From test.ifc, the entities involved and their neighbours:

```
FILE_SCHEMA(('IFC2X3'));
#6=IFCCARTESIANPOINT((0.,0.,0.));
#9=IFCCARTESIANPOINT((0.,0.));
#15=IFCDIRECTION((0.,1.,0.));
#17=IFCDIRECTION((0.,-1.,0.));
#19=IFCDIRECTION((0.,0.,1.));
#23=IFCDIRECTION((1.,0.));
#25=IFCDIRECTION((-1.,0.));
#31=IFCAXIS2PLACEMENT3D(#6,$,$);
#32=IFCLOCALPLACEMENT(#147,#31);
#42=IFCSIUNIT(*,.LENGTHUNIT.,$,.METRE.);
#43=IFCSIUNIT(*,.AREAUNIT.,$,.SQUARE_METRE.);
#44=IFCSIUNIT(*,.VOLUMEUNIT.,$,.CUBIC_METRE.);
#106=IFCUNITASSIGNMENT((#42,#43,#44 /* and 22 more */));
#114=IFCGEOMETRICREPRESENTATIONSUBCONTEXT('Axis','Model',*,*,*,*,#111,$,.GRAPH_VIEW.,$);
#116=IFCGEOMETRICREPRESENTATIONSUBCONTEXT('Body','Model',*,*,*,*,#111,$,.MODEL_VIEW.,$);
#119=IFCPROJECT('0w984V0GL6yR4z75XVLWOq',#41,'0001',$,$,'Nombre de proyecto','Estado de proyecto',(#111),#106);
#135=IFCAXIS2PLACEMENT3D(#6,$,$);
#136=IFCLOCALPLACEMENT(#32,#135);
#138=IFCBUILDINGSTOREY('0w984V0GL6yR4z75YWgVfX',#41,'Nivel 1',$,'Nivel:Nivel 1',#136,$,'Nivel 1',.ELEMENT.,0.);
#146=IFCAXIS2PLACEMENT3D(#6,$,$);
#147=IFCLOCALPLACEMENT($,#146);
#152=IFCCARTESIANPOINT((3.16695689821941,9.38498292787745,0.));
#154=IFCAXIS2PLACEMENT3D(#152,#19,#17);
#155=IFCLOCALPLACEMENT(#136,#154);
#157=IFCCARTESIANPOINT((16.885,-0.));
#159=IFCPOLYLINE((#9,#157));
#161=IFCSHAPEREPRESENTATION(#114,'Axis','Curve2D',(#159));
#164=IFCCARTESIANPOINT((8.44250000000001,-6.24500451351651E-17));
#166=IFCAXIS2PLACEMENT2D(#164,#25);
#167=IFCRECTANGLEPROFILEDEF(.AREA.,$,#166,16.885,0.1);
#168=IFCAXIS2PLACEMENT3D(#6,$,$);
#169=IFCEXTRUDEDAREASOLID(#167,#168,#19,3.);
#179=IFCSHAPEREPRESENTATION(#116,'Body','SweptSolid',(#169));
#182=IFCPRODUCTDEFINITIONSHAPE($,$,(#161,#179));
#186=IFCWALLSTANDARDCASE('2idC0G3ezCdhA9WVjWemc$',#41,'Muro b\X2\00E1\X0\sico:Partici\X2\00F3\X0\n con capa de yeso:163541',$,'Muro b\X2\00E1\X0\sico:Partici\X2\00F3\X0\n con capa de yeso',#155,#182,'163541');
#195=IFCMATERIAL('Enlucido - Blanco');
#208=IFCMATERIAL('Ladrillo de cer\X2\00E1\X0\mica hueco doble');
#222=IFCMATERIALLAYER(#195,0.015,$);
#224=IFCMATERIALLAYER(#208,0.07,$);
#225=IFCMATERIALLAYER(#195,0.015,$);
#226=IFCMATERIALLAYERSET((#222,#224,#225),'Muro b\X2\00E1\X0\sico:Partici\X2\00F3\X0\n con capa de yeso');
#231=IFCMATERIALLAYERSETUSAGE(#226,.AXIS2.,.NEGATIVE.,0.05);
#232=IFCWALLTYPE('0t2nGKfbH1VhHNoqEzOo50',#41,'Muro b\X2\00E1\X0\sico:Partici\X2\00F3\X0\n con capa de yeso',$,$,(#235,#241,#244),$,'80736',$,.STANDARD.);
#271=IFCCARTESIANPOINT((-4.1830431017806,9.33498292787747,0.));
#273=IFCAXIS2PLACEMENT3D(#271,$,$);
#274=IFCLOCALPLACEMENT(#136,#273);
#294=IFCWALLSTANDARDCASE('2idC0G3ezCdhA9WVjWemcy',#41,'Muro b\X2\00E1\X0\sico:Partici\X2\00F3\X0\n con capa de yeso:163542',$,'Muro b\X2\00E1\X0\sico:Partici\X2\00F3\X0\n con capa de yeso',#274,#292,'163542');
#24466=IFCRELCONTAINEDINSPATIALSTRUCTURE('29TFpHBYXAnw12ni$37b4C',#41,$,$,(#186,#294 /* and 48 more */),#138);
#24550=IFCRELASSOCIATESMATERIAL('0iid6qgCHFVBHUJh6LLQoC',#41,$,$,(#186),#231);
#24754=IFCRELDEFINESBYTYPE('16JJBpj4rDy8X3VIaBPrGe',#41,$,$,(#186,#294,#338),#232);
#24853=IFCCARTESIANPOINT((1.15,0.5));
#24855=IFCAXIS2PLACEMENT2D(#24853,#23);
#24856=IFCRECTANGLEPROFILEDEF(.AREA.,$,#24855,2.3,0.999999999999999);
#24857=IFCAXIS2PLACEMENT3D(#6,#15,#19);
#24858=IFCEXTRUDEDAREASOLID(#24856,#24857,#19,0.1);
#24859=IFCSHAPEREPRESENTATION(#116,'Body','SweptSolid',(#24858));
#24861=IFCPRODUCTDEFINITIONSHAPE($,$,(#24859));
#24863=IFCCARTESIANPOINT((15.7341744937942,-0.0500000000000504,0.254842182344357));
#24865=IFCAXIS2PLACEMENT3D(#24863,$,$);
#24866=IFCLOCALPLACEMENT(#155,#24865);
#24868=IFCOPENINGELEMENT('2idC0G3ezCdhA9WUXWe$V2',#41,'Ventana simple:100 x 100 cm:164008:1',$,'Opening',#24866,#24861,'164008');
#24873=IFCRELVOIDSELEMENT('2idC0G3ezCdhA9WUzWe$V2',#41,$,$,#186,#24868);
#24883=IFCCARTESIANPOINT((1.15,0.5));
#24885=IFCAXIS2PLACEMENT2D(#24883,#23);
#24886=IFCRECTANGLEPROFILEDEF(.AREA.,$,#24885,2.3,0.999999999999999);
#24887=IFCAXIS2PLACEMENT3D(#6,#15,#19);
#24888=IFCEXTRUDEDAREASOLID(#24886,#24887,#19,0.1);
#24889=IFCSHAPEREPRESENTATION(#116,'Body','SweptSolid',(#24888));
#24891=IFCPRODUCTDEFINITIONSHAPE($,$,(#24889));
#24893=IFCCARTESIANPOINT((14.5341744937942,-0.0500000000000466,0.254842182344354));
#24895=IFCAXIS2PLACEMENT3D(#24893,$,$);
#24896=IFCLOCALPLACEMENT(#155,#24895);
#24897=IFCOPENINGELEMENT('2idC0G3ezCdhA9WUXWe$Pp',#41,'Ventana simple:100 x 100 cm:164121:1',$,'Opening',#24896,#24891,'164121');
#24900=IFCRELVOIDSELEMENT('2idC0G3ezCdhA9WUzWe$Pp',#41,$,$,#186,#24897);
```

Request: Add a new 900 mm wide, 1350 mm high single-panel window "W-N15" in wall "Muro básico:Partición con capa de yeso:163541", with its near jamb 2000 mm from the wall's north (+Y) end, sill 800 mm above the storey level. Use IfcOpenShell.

```python
import numpy as np
import ifcopenshell
import ifcopenshell.api.feature
import ifcopenshell.api.geometry
import ifcopenshell.api.root
import ifcopenshell.api.spatial
import ifcopenshell.api.type
import ifcopenshell.geom
import ifcopenshell.util.element
import ifcopenshell.util.placement
import ifcopenshell.util.representation
import ifcopenshell.util.shape
import ifcopenshell.util.unit

model = ifcopenshell.open("test.ifc")
unit_scale = ifcopenshell.util.unit.calculate_unit_scale(model)
settings = ifcopenshell.geom.settings()


def volume(element):
    """Net volume in cubic metres, openings subtracted."""
    shape = ifcopenshell.geom.create_shape(settings, element)
    return ifcopenshell.util.shape.get_volume(shape.geometry)


wall = model.by_id(186)
storey = ifcopenshell.util.element.get_container(wall, ifc_class="IfcBuildingStorey")
context = ifcopenshell.util.representation.get_context(model, "Model", "Body", "MODEL_VIEW")
before = volume(wall)

width, height, from_end, sill = 0.9, 1.35, 2, 0.8  # metres

# The wall runs along its own X axis, and the end named is its -X end.
wall_shape = ifcopenshell.geom.create_shape(settings, wall)
x, y, z = ifcopenshell.util.shape.get_vertices(wall_shape.geometry).T
start = x.min() + from_end
face, thickness = float(y.min()), float(y.max() - y.min())
wall_matrix = ifcopenshell.util.placement.get_local_placement(wall.ObjectPlacement)
level = ifcopenshell.util.placement.get_local_placement(storey.ObjectPlacement)[2, 3]


def in_wall(x, y):
    """Placement at x, y metres in the wall's axes, at sill height."""
    matrix = wall_matrix.copy()
    matrix[:, 3] = wall_matrix @ np.array([x / unit_scale, y / unit_scale, 0.0, 1.0])
    matrix[2, 3] = level + sill / unit_scale
    return matrix


# Opening: a box that overshoots both wall faces by 50 mm.
opening = ifcopenshell.api.root.create_entity(model, ifc_class="IfcOpeningElement")
box = ifcopenshell.api.geometry.add_wall_representation(
    model, context=context, length=width, height=height, thickness=thickness + 0.1
)
ifcopenshell.api.geometry.assign_representation(model, product=opening, representation=box)
ifcopenshell.api.geometry.edit_object_placement(model, product=opening, matrix=in_wall(start, face - 0.05), is_si=False)
ifcopenshell.api.feature.add_feature(model, feature=opening, element=wall)

window = ifcopenshell.api.root.create_entity(model, ifc_class="IfcWindow", name="W-N15")
window.OverallWidth, window.OverallHeight = width / unit_scale, height / unit_scale
body = ifcopenshell.api.geometry.add_window_representation(
    model,
    context=context,
    overall_width=window.OverallWidth,
    overall_height=window.OverallHeight,
    partition_type="SINGLE_PANEL",
)
ifcopenshell.api.geometry.assign_representation(model, product=window, representation=body)
ifcopenshell.api.spatial.assign_container(model, products=[window], relating_structure=storey)
fills = ifcopenshell.api.feature.add_filling(model, opening=opening, element=window)
fills.OwnerHistory = window.OwnerHistory  # required in IFC2X3

# IFC2X3 keeps the operation on the window style.
style = ifcopenshell.api.root.create_entity(model, ifc_class="IfcWindowStyle", name="W-N15")
style.OperationType, style.ConstructionType = "SINGLE_PANEL", "NOTDEFINED"
style.ParameterTakesPrecedence = style.Sizeable = False
ifcopenshell.api.type.assign_type(model, related_objects=[window], relating_type=style)

# Centre the window in the wall's thickness.
ifcopenshell.api.geometry.edit_object_placement(model, product=window, matrix=in_wall(start, face), is_si=False)
window_shape = ifcopenshell.geom.create_shape(settings, window)
depth = ifcopenshell.util.shape.get_vertices(window_shape.geometry)[:, 1]
offset = face + thickness / 2 - (depth.min() + depth.max()) / 2
ifcopenshell.api.geometry.edit_object_placement(model, product=window, matrix=in_wall(start, offset), is_si=False)

after = volume(wall)

print(f"wall volume {before:.3f} -> {after:.3f} m3")

model.write("test_edited.ifc")
```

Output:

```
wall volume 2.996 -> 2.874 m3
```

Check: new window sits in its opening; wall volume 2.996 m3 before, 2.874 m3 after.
